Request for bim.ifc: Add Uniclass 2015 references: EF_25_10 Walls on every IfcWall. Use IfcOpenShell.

First a look at what the model holds.

```python
import ifcopenshell

model = ifcopenshell.open("bim.ifc")
print(model.schema)
print("classifications:", [c.Name for c in model.by_type("IfcClassification")])
for ifc_class in ("IfcDoor", "IfcRoof", "IfcStair", "IfcWall", "IfcWindow"):
    print(ifc_class, len(model.by_type(ifc_class)))
```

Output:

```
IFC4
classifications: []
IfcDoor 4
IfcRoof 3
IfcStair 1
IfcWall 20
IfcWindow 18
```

```python
import ifcopenshell
import ifcopenshell.api.classification

model = ifcopenshell.open("bim.ifc")

system = ifcopenshell.api.classification.add_classification(model, classification="Uniclass 2015")

codes = {
    "IfcWall": ("EF_25_10", "Walls"),
}
for ifc_class, (code, name) in codes.items():
    products = model.by_type(ifc_class)
    ifcopenshell.api.classification.add_reference(
        model, products=products, classification=system, identification=code, name=name
    )
    print(code, len(products))

model.write("bim_edited.ifc")
```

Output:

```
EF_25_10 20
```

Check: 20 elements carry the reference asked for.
